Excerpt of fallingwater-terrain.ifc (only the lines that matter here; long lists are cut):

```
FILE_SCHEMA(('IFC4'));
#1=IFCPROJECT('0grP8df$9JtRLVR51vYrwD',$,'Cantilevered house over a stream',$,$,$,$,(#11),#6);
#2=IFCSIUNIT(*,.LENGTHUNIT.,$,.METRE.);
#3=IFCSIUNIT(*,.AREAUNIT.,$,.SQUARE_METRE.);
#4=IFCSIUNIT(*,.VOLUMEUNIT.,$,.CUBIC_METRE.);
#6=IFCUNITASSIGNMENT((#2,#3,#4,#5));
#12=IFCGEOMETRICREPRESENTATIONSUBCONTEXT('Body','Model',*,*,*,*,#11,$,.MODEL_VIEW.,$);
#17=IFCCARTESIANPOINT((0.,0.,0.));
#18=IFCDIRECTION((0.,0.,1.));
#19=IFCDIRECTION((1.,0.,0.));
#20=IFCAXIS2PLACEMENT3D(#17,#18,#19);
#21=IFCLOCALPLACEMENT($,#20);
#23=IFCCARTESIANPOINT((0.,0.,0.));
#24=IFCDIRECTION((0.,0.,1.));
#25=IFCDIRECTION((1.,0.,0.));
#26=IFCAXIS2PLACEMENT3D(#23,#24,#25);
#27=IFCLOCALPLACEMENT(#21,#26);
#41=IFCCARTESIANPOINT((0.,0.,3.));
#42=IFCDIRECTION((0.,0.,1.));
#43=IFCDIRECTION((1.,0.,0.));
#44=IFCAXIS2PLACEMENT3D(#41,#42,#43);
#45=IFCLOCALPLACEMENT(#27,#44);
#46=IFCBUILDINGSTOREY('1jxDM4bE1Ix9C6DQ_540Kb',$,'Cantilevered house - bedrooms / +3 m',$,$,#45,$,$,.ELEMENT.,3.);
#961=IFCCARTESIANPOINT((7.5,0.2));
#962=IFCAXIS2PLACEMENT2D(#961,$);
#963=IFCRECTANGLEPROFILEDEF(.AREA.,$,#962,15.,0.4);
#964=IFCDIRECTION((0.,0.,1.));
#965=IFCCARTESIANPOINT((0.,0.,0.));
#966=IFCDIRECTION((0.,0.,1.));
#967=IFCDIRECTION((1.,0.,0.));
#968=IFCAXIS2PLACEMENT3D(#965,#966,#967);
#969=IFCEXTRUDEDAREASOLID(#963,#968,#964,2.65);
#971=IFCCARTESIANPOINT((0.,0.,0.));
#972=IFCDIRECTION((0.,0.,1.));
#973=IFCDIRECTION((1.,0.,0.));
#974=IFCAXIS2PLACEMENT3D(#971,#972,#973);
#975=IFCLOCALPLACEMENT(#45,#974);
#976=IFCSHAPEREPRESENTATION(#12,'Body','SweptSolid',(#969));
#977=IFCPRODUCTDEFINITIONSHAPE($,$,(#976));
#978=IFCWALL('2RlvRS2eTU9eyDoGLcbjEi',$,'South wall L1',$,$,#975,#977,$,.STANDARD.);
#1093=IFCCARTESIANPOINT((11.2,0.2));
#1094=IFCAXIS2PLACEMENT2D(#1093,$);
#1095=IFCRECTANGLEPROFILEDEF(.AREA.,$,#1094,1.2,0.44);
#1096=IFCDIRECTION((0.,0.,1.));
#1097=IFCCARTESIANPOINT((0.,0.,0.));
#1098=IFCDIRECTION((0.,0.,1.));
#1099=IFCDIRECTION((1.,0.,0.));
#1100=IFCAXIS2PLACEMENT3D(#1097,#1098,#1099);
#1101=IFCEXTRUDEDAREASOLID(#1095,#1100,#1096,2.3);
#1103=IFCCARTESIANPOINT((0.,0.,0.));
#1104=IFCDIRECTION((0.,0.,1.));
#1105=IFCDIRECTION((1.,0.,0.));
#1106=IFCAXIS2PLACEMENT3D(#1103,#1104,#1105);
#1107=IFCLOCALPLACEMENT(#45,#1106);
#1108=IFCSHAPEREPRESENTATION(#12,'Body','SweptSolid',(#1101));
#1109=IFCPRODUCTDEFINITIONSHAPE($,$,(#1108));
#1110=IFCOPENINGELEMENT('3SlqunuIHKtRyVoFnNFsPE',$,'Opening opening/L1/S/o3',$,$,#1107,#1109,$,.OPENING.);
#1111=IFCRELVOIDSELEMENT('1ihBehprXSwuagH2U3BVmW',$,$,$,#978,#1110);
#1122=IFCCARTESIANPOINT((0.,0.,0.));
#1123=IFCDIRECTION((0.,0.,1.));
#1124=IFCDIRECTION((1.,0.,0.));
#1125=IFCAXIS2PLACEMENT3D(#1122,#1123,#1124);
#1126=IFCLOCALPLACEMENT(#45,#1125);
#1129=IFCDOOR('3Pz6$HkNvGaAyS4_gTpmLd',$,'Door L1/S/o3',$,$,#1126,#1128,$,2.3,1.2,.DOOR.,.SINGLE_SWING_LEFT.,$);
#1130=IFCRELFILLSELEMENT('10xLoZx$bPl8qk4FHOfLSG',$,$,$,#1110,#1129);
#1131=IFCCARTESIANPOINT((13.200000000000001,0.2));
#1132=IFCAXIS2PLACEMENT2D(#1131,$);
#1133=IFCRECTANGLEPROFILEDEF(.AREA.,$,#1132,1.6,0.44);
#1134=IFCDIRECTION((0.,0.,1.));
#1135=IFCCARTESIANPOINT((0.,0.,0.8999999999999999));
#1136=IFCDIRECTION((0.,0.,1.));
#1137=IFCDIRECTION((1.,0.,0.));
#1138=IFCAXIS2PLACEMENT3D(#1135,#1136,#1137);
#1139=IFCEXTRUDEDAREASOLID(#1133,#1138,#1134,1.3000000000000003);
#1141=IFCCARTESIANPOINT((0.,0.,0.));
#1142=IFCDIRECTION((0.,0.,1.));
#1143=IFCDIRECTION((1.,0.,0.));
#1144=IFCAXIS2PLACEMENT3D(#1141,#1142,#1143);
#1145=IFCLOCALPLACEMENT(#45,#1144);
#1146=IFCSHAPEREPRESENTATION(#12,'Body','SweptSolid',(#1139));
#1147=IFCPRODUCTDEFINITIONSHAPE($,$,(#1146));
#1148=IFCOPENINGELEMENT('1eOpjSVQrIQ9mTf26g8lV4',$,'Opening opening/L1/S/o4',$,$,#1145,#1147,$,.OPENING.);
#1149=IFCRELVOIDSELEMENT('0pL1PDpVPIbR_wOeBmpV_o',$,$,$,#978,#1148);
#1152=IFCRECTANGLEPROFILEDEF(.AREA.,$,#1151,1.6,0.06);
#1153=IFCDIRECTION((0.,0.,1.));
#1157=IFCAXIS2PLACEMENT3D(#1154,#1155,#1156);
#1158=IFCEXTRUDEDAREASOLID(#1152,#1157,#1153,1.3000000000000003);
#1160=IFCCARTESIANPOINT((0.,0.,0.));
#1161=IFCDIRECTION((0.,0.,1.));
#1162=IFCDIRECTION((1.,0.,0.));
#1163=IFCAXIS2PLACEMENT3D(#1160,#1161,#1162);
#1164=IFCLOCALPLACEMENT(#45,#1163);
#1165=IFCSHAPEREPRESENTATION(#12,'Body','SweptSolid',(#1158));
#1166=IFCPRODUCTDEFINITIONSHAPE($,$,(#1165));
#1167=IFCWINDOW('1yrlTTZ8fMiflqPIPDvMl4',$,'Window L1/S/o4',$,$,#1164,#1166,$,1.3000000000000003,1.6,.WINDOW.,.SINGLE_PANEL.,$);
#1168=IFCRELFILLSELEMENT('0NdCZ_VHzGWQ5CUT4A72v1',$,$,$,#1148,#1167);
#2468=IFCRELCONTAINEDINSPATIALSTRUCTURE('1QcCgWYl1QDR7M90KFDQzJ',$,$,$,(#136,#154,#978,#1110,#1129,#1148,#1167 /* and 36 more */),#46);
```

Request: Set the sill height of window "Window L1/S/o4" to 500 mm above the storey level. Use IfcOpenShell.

```python
import numpy as np
import ifcopenshell
import ifcopenshell.api.geometry
import ifcopenshell.geom
import ifcopenshell.util.element
import ifcopenshell.util.placement
import ifcopenshell.util.shape
import ifcopenshell.util.unit

model = ifcopenshell.open("fallingwater-terrain.ifc")
unit_scale = ifcopenshell.util.unit.calculate_unit_scale(model)

window = model.by_guid("1yrlTTZ8fMiflqPIPDvMl4")
opening = window.FillsVoids[0].RelatingOpeningElement
storey = ifcopenshell.util.element.get_container(window, ifc_class="IfcBuildingStorey")
level = ifcopenshell.util.placement.get_local_placement(storey.ObjectPlacement)[2, 3]

# The opening's origin need not be at the sill, so measure its lowest point.
shape = ifcopenshell.geom.create_shape(ifcopenshell.geom.settings(), opening)
bottom = ifcopenshell.util.shape.get_shape_bottom_elevation(shape, shape.geometry) / unit_scale
dz = level + 0.5 / unit_scale - bottom

shift = np.array([0.0, 0.0, dz])
# The window is not placed relative to its opening, so move both.
for product in (opening, window):
    matrix = ifcopenshell.util.placement.get_local_placement(product.ObjectPlacement)
    matrix[:3, 3] += shift
    ifcopenshell.api.geometry.edit_object_placement(model, product=product, matrix=matrix, is_si=False)

print(f"moved by {dz * unit_scale:+.3f} m")

model.write("fallingwater-terrain-out.ifc")
```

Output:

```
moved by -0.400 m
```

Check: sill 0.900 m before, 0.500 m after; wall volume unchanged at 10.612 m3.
